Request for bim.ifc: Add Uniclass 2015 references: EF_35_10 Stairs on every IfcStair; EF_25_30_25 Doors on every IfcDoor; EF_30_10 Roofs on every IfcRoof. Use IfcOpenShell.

First a look at what the model holds.

```python
import ifcopenshell

model = ifcopenshell.open("bim.ifc")
print(model.schema)
print("classifications:", [c.Name for c in model.by_type("IfcClassification")])
for ifc_class in ("IfcDoor", "IfcRoof", "IfcStair", "IfcWall", "IfcWindow"):
    print(ifc_class, len(model.by_type(ifc_class)))
```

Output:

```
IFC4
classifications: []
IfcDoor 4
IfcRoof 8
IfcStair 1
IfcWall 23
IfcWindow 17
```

```python
import ifcopenshell
import ifcopenshell.api.classification

model = ifcopenshell.open("bim.ifc")

system = ifcopenshell.api.classification.add_classification(model, classification="Uniclass 2015")

codes = {
    "IfcStair": ("EF_35_10", "Stairs"),
    "IfcDoor": ("EF_25_30_25", "Doors"),
    "IfcRoof": ("EF_30_10", "Roofs"),
}
for ifc_class, (code, name) in codes.items():
    products = model.by_type(ifc_class)
    ifcopenshell.api.classification.add_reference(
        model, products=products, classification=system, identification=code, name=name
    )
    print(code, len(products))

model.write("bim_rev.ifc")
```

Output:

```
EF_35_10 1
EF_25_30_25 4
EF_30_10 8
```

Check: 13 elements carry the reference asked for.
